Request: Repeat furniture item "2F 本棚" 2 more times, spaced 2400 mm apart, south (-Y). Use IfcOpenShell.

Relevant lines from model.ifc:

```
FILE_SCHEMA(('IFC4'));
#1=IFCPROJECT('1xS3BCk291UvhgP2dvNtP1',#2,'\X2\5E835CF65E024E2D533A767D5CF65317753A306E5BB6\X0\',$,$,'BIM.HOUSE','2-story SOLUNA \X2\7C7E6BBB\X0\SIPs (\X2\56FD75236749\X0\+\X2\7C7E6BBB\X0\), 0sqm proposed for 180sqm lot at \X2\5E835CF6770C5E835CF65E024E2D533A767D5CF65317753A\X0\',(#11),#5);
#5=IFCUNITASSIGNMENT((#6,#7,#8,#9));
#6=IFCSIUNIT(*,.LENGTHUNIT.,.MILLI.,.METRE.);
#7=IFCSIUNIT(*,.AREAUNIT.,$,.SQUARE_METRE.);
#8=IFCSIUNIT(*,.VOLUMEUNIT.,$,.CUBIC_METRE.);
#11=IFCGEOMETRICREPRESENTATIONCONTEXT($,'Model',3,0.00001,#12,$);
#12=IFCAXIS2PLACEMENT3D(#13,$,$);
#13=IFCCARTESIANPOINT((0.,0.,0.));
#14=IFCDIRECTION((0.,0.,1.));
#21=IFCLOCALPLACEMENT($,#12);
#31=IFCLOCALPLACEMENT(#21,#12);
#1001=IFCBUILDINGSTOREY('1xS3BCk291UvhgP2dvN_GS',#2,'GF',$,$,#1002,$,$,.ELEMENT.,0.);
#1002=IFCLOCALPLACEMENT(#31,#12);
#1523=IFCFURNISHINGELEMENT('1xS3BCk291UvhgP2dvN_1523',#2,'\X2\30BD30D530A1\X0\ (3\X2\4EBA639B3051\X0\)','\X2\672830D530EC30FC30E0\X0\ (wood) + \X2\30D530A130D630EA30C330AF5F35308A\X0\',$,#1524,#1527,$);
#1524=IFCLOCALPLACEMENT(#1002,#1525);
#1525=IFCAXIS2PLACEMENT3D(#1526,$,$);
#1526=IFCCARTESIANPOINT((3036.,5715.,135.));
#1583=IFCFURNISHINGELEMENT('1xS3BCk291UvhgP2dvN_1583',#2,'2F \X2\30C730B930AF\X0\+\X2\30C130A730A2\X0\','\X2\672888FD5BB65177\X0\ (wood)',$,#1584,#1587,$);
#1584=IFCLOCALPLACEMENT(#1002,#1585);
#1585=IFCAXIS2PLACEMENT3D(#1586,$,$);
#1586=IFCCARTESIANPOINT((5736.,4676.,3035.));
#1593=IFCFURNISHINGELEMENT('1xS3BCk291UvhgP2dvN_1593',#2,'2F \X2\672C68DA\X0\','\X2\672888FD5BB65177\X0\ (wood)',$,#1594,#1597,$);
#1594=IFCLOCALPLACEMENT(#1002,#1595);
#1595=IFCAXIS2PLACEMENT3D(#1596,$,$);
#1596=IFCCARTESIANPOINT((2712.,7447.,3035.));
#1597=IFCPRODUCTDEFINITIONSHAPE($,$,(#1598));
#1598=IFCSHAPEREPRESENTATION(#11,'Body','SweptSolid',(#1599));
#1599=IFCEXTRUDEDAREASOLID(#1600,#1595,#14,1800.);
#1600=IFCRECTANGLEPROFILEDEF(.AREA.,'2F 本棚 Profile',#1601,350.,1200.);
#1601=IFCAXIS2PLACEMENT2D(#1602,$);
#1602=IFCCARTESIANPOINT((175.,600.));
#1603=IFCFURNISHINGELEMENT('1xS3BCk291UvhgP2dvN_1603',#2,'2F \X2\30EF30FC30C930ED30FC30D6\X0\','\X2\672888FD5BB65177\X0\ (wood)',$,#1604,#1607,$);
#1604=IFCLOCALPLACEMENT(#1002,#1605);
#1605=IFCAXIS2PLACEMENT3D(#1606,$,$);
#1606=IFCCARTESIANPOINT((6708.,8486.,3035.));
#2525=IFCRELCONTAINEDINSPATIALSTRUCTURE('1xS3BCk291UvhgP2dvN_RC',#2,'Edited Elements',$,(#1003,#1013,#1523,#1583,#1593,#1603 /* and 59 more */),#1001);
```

```python
import numpy as np
import ifcopenshell
import ifcopenshell.api.geometry
import ifcopenshell.api.root
import ifcopenshell.util.element
import ifcopenshell.util.placement

model = ifcopenshell.open("model.ifc")


def reuse_history(source, copy):
    """copy_class also copies each property set's owner history, people and application; keep the originals."""
    for rel in copy.IsDefinedBy:
        if rel.is_a("IfcRelDefinesByProperties") and (history := rel.RelatingPropertyDefinition.OwnerHistory):
            rel.RelatingPropertyDefinition.OwnerHistory = source.OwnerHistory
            ifcopenshell.util.element.remove_deep2(model, history)


source = model.by_guid("1xS3BCk291UvhgP2dvN_1593")
base = ifcopenshell.util.placement.get_local_placement(source.ObjectPlacement)
step = np.array([0.0, -1.0, 0.0]) * 2400.0

for i in range(1, 3):
    copy = ifcopenshell.api.root.copy_class(model, product=source)
    copy.Representation = ifcopenshell.util.element.copy_deep(
        model, source.Representation, exclude=["IfcGeometricRepresentationContext", "IfcRepresentationMap"]
    )
    reuse_history(source, copy)
    matrix = base.copy()
    matrix[:3, 3] += i * step
    print("added at", matrix[:3, 3].round(3) + 0.0)
    ifcopenshell.api.geometry.edit_object_placement(model, product=copy, matrix=matrix, is_si=False)

model.write("model_rev.ifc")
```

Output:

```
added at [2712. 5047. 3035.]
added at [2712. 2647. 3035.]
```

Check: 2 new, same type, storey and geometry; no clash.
